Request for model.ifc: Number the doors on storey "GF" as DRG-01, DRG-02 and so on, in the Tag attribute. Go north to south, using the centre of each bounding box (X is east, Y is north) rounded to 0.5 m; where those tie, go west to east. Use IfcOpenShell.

First a look at what the model holds.

```python
import ifcopenshell
import ifcopenshell.util.element
import ifcopenshell.util.placement

model = ifcopenshell.open("model.ifc")
print(model.schema)
storey = next(s for s in model.by_type("IfcBuildingStorey") if s.Name == "GF")
doors = [e for e in ifcopenshell.util.element.get_decomposition(storey) if e.is_a("IfcDoor")]
for e in sorted(doors, key=lambda e: e.id()):
    origin = ifcopenshell.util.placement.get_local_placement(e.ObjectPlacement)[:3, 3]
    print(e.id(), e.Tag, e.Name, origin.round(2) + 0.0, sep=" | ")
```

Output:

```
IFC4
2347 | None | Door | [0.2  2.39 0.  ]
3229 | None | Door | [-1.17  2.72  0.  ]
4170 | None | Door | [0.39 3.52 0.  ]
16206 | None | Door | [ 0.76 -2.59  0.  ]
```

```python
import ifcopenshell
import ifcopenshell.geom
import ifcopenshell.util.element
import ifcopenshell.util.shape

model = ifcopenshell.open("model.ifc")
settings = ifcopenshell.geom.settings()
settings.set("use-world-coords", True)


def centre(element):
    shape = ifcopenshell.geom.create_shape(settings, element)
    return ifcopenshell.util.shape.get_bbox_centroid(shape.geometry)


storey = next(s for s in model.by_type("IfcBuildingStorey") if s.Name == "GF")
doors = [e for e in ifcopenshell.util.element.get_decomposition(storey) if e.is_a("IfcDoor")]

# Insertion points can sit at a corner or the storey origin, so sort by the geometry (in metres).
centres = {e: centre(e) for e in doors}
doors.sort(key=lambda e: (-round(centres[e][1] / 0.5), centres[e][0]))

for i, e in enumerate(doors, start=1):
    number = f"DRG-{i:02d}"
    e.Tag = number
    print(e.id(), number)

model.write("model-out.ifc")
```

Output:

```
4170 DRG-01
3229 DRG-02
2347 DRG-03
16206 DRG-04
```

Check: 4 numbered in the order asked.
